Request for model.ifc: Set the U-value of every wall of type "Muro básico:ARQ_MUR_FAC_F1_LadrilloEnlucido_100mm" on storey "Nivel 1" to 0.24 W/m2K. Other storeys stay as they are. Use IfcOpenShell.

First a look at what the model holds.

```python
import ifcopenshell
import ifcopenshell.util.element

model = ifcopenshell.open("model.ifc")
print(model.schema)
storey = next(s for s in model.by_type("IfcBuildingStorey") if s.Name == "Nivel 1")
walls = [e for e in ifcopenshell.util.element.get_decomposition(storey) if e.is_a("IfcWall")]
seen = {}
for e in walls:
    element_type = ifcopenshell.util.element.get_type(e)
    key = (element_type.Name if element_type != e and element_type else None, ifcopenshell.util.element.get_pset(e, "Pset_WallCommon", "ThermalTransmittance"))
    seen[key] = seen.get(key, 0) + 1
for (name, value), count in sorted(seen.items(), key=str):
    print(count, "x", name, "|", value)
```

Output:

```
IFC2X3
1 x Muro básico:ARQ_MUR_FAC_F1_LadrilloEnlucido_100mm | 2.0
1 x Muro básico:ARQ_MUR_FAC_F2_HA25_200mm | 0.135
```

```python
import ifcopenshell
import ifcopenshell.api.pset
import ifcopenshell.util.element

model = ifcopenshell.open("model.ifc")

storey = next(s for s in model.by_type("IfcBuildingStorey") if s.Name == "Nivel 1")
walls = [e for e in ifcopenshell.util.element.get_decomposition(storey) if e.is_a("IfcWall")]

count = 0
for e in walls:
    element_type = ifcopenshell.util.element.get_type(e)
    if element_type in (None, e) or element_type.Name != "Muro básico:ARQ_MUR_FAC_F1_LadrilloEnlucido_100mm":
        continue
    # add_pset returns the element's existing set when there is one.
    pset = ifcopenshell.api.pset.add_pset(model, product=e, name="Pset_WallCommon")
    ifcopenshell.api.pset.edit_pset(model, pset=pset, properties={"ThermalTransmittance": 0.24})
    count += 1

print(count, "walls updated")

model.write("model-out.ifc")
```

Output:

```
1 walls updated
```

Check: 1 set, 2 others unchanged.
